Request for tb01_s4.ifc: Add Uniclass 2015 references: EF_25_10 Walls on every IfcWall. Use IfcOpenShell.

First a look at what the model holds.

```python
import ifcopenshell

model = ifcopenshell.open("tb01_s4.ifc")
print(model.schema)
print("classifications:", [c.Name for c in model.by_type("IfcClassification")])
for ifc_class in ("IfcDoor", "IfcRoof", "IfcStair", "IfcWall", "IfcWindow"):
    print(ifc_class, len(model.by_type(ifc_class)))
```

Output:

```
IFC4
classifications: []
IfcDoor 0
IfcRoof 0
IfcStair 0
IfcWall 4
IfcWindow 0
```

```python
import ifcopenshell
import ifcopenshell.api.classification

model = ifcopenshell.open("tb01_s4.ifc")

system = ifcopenshell.api.classification.add_classification(model, classification="Uniclass 2015")

codes = {
    "IfcWall": ("EF_25_10", "Walls"),
}
for ifc_class, (code, name) in codes.items():
    products = model.by_type(ifc_class)
    ifcopenshell.api.classification.add_reference(
        model, products=products, classification=system, identification=code, name=name
    )
    print(code, len(products))

model.write("tb01_s4_updated.ifc")
```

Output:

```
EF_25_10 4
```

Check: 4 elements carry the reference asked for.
